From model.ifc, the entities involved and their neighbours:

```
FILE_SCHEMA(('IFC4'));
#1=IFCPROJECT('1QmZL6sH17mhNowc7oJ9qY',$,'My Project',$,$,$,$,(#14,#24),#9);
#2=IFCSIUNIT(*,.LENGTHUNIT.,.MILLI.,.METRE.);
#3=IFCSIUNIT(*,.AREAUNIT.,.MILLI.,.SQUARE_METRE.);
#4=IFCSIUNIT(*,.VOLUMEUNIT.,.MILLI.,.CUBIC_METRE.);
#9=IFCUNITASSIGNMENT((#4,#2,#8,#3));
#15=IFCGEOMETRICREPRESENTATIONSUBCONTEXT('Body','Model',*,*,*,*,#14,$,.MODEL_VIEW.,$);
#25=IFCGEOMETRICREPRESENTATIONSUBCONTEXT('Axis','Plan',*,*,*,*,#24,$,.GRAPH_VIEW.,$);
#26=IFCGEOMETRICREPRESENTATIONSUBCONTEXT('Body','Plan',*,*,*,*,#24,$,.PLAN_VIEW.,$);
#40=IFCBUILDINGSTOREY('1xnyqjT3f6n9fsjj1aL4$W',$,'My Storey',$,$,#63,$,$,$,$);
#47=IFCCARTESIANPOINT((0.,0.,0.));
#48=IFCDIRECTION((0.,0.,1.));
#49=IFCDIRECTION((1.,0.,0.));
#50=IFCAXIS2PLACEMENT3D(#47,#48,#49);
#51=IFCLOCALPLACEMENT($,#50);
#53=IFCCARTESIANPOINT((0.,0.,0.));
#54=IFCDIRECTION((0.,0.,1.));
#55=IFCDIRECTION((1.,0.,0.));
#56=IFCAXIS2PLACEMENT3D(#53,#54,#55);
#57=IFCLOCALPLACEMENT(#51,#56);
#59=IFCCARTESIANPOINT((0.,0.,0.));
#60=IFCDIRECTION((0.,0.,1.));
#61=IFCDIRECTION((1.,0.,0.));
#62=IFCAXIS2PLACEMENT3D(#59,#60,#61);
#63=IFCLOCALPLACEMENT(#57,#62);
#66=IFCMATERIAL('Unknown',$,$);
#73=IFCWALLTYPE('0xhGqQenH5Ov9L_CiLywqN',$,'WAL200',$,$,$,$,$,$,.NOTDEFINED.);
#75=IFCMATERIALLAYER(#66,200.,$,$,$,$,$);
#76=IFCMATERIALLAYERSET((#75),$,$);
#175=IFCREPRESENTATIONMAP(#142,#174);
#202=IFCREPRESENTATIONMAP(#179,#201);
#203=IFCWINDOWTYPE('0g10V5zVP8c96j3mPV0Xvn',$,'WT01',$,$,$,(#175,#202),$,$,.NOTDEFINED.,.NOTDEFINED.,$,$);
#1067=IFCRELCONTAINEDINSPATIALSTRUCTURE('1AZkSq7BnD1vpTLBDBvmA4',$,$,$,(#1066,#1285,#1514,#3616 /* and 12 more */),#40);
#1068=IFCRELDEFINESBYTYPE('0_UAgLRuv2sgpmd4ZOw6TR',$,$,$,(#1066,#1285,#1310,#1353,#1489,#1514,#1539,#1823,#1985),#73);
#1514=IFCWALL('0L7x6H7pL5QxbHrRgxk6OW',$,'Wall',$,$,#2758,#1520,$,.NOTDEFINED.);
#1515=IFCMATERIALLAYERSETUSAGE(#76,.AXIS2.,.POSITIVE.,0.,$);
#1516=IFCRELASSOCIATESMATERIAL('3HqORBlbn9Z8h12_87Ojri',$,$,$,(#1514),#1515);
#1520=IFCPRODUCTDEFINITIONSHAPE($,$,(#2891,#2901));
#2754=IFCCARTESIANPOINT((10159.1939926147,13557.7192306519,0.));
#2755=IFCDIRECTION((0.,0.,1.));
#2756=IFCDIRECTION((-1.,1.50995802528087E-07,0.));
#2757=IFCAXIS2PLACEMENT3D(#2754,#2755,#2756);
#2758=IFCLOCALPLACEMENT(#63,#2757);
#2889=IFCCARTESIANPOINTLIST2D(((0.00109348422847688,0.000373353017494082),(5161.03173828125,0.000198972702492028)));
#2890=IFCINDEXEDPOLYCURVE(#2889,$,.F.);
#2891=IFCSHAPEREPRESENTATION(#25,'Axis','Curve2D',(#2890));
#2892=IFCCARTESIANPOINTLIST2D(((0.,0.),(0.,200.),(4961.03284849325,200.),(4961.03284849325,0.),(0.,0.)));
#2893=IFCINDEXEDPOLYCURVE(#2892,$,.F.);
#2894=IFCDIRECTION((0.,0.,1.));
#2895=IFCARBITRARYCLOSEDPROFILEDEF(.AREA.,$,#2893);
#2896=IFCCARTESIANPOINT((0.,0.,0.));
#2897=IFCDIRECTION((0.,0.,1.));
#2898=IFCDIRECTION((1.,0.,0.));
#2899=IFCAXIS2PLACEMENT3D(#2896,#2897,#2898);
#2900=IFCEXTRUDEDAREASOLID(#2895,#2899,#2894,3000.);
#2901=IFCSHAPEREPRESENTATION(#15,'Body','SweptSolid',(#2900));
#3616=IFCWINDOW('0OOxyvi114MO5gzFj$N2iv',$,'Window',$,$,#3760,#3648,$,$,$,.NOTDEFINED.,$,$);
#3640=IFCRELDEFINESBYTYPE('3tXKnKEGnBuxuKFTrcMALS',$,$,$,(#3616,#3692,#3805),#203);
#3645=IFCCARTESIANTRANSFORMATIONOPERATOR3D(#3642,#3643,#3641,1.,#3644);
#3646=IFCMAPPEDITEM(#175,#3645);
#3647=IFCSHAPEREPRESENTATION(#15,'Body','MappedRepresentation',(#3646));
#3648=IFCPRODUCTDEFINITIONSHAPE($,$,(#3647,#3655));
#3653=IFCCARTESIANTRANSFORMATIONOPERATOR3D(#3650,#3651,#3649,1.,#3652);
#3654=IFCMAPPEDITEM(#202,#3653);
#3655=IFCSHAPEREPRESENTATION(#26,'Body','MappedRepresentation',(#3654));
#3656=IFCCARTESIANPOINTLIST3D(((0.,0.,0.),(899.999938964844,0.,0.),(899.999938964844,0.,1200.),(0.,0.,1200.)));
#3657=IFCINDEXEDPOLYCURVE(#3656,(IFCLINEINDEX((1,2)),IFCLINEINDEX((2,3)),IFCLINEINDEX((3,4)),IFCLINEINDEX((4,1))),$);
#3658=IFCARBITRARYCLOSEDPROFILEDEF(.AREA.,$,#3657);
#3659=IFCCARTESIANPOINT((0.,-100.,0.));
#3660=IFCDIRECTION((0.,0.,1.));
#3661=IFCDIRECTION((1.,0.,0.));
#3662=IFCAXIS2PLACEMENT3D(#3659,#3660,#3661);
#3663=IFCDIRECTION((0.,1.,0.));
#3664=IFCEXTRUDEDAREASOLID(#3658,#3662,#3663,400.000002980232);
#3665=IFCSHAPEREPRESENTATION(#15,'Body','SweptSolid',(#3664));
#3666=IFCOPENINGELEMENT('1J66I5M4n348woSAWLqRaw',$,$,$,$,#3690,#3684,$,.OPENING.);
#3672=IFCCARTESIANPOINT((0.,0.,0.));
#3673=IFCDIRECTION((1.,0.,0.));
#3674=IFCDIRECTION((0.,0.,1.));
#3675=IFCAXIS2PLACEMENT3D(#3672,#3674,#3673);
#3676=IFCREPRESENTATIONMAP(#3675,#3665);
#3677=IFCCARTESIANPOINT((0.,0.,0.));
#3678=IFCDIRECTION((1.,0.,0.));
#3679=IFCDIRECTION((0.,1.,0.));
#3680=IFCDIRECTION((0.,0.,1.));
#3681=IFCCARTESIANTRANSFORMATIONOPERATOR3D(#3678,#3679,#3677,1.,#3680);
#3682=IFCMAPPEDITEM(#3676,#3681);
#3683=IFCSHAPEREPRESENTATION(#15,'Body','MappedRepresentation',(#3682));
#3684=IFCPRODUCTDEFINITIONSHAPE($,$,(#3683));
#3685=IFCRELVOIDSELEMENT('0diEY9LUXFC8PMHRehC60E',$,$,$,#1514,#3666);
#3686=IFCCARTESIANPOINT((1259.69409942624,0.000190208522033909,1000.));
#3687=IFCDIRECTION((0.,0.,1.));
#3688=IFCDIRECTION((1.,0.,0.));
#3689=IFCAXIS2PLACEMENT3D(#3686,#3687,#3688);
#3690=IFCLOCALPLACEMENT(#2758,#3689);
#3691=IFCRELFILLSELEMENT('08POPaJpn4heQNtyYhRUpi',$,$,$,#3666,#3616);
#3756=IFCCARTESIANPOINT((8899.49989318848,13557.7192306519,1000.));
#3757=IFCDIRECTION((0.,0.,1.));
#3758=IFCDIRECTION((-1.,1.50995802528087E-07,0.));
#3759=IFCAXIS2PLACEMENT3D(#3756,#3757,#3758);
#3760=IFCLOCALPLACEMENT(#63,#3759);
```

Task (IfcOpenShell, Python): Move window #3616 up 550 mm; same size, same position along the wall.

```python
import numpy as np
import ifcopenshell
import ifcopenshell.api.geometry
import ifcopenshell.util.placement
import ifcopenshell.util.unit

model = ifcopenshell.open("model.ifc")
unit_scale = ifcopenshell.util.unit.calculate_unit_scale(model)

window = model.by_guid("0OOxyvi114MO5gzFj$N2iv")
opening = window.FillsVoids[0].RelatingOpeningElement
dz = 0.55 / unit_scale

shift = np.array([0.0, 0.0, dz])
# The window is not placed relative to its opening, so move both.
for product in (opening, window):
    matrix = ifcopenshell.util.placement.get_local_placement(product.ObjectPlacement)
    matrix[:3, 3] += shift
    ifcopenshell.api.geometry.edit_object_placement(model, product=product, matrix=matrix, is_si=False)

print(f"moved by {dz * unit_scale:+.3f} m")

model.write("model_rev.ifc")
```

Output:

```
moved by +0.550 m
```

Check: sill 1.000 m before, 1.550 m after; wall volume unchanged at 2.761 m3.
